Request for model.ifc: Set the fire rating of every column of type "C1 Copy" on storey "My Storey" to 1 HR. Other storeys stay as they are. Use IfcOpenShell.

First a look at what the model holds.

```python
import ifcopenshell
import ifcopenshell.util.element

model = ifcopenshell.open("model.ifc")
print(model.schema)
storey = next(s for s in model.by_type("IfcBuildingStorey") if s.Name == "My Storey")
columns = [e for e in ifcopenshell.util.element.get_decomposition(storey) if e.is_a("IfcColumn")]
seen = {}
for e in columns:
    element_type = ifcopenshell.util.element.get_type(e)
    key = (element_type.Name if element_type != e and element_type else None, ifcopenshell.util.element.get_pset(e, "Pset_ColumnCommon", "FireRating"))
    seen[key] = seen.get(key, 0) + 1
for (name, value), count in sorted(seen.items(), key=str):
    print(count, "x", name, "|", value)
```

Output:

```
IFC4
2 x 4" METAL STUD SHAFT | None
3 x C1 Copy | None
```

```python
import ifcopenshell
import ifcopenshell.api.pset
import ifcopenshell.util.element

model = ifcopenshell.open("model.ifc")

storey = next(s for s in model.by_type("IfcBuildingStorey") if s.Name == "My Storey")
columns = [e for e in ifcopenshell.util.element.get_decomposition(storey) if e.is_a("IfcColumn")]

count = 0
for e in columns:
    element_type = ifcopenshell.util.element.get_type(e)
    if element_type in (None, e) or element_type.Name != "C1 Copy":
        continue
    # add_pset returns the element's existing set when there is one.
    pset = ifcopenshell.api.pset.add_pset(model, product=e, name="Pset_ColumnCommon")
    ifcopenshell.api.pset.edit_pset(model, pset=pset, properties={"FireRating": "1 HR"})
    count += 1

print(count, "columns updated")

model.write("model_v2.ifc")
```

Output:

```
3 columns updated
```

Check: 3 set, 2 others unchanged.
